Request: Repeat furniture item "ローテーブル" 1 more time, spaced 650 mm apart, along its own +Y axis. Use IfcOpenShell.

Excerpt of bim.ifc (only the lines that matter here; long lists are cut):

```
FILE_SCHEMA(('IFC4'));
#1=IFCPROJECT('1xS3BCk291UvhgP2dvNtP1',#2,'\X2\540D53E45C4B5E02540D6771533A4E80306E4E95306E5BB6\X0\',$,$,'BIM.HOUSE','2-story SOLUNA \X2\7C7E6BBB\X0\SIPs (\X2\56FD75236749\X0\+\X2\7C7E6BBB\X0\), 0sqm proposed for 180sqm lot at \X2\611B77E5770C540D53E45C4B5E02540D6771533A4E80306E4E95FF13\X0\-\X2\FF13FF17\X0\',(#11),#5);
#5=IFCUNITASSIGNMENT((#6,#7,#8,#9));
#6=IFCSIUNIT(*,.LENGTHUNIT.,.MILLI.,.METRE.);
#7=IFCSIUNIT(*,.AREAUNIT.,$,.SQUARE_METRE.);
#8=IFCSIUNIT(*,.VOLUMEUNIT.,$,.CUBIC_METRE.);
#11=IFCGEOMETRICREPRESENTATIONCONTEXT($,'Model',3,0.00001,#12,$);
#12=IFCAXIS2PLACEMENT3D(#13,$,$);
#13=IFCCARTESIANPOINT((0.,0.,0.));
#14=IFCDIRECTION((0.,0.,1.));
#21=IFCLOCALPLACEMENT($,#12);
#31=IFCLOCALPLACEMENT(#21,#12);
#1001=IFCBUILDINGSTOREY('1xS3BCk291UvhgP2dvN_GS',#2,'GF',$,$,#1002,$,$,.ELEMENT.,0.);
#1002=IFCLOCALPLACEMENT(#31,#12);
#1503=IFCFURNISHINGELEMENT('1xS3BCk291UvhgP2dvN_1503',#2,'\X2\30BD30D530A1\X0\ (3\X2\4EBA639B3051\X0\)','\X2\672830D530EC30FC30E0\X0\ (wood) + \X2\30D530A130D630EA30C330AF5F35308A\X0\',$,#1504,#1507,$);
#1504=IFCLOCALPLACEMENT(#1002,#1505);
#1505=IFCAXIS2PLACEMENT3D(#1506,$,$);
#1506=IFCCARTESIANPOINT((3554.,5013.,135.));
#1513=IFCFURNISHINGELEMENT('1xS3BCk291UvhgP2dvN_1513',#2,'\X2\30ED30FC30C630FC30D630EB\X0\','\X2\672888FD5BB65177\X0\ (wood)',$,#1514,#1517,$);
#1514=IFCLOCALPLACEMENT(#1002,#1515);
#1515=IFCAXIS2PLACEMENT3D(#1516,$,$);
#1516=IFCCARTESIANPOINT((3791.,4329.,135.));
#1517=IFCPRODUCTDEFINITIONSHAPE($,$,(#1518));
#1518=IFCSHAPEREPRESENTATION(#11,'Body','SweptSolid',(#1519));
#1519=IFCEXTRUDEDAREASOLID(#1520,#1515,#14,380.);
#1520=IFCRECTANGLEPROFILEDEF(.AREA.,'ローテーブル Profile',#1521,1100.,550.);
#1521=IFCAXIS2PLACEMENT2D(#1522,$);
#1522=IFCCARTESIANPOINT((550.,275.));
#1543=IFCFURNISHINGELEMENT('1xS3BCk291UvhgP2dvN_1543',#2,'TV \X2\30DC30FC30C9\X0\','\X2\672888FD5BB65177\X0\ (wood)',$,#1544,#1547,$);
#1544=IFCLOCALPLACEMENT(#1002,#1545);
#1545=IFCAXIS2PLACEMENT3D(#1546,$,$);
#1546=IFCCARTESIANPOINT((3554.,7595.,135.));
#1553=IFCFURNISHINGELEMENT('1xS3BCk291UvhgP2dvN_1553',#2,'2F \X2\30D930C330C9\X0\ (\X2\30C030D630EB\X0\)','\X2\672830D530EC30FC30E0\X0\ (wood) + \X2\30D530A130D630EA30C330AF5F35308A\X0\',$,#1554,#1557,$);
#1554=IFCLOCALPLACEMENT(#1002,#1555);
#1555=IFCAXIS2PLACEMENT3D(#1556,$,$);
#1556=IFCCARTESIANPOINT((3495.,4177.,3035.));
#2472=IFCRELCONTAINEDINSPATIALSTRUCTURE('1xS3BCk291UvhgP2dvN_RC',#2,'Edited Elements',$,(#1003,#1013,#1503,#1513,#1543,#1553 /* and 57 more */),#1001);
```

```python
import ifcopenshell
import ifcopenshell.api.geometry
import ifcopenshell.api.root
import ifcopenshell.util.element
import ifcopenshell.util.placement

model = ifcopenshell.open("bim.ifc")


def reuse_history(source, copy):
    """copy_class also copies each property set's owner history, people and application; keep the originals."""
    for rel in copy.IsDefinedBy:
        if rel.is_a("IfcRelDefinesByProperties") and (history := rel.RelatingPropertyDefinition.OwnerHistory):
            rel.RelatingPropertyDefinition.OwnerHistory = source.OwnerHistory
            ifcopenshell.util.element.remove_deep2(model, history)


source = model.by_guid("1xS3BCk291UvhgP2dvN_1513")
base = ifcopenshell.util.placement.get_local_placement(source.ObjectPlacement)
step = base[:3, 1] * 650.0

for i in range(1, 2):
    copy = ifcopenshell.api.root.copy_class(model, product=source)
    copy.Representation = ifcopenshell.util.element.copy_deep(
        model, source.Representation, exclude=["IfcGeometricRepresentationContext", "IfcRepresentationMap"]
    )
    reuse_history(source, copy)
    matrix = base.copy()
    matrix[:3, 3] += i * step
    print("added at", matrix[:3, 3].round(3) + 0.0)
    ifcopenshell.api.geometry.edit_object_placement(model, product=copy, matrix=matrix, is_si=False)

model.write("bim_v2.ifc")
```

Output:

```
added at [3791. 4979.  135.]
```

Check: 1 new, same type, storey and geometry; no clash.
